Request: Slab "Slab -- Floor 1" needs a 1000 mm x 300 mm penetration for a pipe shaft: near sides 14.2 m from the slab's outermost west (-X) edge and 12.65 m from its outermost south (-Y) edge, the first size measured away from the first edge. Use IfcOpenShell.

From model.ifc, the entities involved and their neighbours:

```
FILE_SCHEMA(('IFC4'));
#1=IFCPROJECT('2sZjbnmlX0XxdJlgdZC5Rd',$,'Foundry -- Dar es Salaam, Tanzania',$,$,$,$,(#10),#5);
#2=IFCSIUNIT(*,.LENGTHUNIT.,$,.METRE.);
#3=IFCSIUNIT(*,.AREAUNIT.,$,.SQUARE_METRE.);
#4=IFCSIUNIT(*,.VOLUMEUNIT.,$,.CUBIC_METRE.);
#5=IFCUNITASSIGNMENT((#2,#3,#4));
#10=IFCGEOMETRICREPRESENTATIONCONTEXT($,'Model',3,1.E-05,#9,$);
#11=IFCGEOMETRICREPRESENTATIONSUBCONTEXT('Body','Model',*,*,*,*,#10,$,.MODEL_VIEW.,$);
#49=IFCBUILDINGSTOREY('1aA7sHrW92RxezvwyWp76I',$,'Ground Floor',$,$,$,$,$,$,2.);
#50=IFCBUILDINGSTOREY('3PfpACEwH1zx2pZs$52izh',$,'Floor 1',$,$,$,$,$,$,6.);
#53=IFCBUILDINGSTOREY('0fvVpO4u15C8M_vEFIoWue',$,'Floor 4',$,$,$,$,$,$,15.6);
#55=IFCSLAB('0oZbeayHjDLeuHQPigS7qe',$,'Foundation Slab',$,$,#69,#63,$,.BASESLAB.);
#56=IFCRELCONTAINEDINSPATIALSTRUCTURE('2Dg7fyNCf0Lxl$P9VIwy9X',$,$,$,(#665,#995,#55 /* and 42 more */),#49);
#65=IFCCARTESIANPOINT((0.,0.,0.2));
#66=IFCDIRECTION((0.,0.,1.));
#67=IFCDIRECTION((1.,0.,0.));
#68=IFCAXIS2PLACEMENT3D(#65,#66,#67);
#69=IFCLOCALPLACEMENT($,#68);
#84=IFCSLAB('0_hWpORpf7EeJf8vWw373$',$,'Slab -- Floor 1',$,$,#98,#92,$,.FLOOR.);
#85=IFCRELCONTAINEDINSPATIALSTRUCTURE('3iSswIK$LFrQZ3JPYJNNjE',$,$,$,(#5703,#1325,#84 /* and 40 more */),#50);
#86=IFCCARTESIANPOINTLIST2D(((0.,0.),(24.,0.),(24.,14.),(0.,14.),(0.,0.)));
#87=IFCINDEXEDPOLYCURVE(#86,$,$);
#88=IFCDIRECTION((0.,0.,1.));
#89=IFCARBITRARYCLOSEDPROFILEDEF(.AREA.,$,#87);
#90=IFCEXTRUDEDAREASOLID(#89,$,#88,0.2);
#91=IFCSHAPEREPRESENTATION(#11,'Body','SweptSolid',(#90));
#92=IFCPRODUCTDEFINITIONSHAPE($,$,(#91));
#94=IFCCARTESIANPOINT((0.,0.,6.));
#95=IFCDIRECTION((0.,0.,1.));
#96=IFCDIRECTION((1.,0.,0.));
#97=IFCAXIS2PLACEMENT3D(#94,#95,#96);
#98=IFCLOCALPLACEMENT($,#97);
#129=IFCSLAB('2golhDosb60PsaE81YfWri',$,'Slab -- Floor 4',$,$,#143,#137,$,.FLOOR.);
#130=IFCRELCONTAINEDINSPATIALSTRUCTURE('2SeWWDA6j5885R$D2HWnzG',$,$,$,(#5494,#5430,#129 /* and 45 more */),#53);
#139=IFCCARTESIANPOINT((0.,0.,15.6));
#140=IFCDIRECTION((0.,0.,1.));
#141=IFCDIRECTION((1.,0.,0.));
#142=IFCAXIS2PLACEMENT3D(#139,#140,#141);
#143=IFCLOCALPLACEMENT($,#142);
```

```python
import numpy as np
import ifcopenshell
import ifcopenshell.api.feature
import ifcopenshell.api.geometry
import ifcopenshell.api.root
import ifcopenshell.geom
import ifcopenshell.util.placement
import ifcopenshell.util.representation
import ifcopenshell.util.shape
import ifcopenshell.util.unit

model = ifcopenshell.open("model.ifc")
unit_scale = ifcopenshell.util.unit.calculate_unit_scale(model)
settings = ifcopenshell.geom.settings()


def volume(element):
    """Net volume in cubic metres, openings subtracted."""
    shape = ifcopenshell.geom.create_shape(settings, element)
    return ifcopenshell.util.shape.get_volume(shape.geometry)


slab = model.by_guid("0_hWpORpf7EeJf8vWw373$")
before = volume(slab)

# Extent in the slab's own axes, in metres. The edges named are its -X and -Y sides.
slab_shape = ifcopenshell.geom.create_shape(settings, slab)
vertices = ifcopenshell.util.shape.get_vertices(slab_shape.geometry)
x_min, y_min, bottom = vertices.min(axis=0)
top = vertices[:, 2].max()

opening = ifcopenshell.api.root.create_entity(model, ifc_class="IfcOpeningElement", name="Pipe shaft opening", predefined_type="OPENING")
context = ifcopenshell.util.representation.get_context(model, "Model", "Body", "MODEL_VIEW")
width, depth = 1, 0.3
outline = [(0.0, 0.0), (width, 0.0), (width, depth), (0.0, depth), (0.0, 0.0)]
# Overshoot both faces by 50 mm so the cut is clean.
shape = ifcopenshell.api.geometry.add_slab_representation(
    model, context=context, depth=top - bottom + 0.1, polyline=outline
)
ifcopenshell.api.geometry.assign_representation(model, product=opening, representation=shape)

matrix = ifcopenshell.util.placement.get_local_placement(slab.ObjectPlacement)
matrix[:, 3] = matrix @ np.append(np.array([x_min + 14.2, y_min + 12.65, bottom - 0.05]) / unit_scale, 1.0)
ifcopenshell.api.geometry.edit_object_placement(model, product=opening, matrix=matrix, is_si=False)
ifcopenshell.api.feature.add_feature(model, feature=opening, element=slab)

after = volume(slab)

print(f"slab volume {before:.3f} -> {after:.3f} m3")

model.write("model_updated.ifc")
```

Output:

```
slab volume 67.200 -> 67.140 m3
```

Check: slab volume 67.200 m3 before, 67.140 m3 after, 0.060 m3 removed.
